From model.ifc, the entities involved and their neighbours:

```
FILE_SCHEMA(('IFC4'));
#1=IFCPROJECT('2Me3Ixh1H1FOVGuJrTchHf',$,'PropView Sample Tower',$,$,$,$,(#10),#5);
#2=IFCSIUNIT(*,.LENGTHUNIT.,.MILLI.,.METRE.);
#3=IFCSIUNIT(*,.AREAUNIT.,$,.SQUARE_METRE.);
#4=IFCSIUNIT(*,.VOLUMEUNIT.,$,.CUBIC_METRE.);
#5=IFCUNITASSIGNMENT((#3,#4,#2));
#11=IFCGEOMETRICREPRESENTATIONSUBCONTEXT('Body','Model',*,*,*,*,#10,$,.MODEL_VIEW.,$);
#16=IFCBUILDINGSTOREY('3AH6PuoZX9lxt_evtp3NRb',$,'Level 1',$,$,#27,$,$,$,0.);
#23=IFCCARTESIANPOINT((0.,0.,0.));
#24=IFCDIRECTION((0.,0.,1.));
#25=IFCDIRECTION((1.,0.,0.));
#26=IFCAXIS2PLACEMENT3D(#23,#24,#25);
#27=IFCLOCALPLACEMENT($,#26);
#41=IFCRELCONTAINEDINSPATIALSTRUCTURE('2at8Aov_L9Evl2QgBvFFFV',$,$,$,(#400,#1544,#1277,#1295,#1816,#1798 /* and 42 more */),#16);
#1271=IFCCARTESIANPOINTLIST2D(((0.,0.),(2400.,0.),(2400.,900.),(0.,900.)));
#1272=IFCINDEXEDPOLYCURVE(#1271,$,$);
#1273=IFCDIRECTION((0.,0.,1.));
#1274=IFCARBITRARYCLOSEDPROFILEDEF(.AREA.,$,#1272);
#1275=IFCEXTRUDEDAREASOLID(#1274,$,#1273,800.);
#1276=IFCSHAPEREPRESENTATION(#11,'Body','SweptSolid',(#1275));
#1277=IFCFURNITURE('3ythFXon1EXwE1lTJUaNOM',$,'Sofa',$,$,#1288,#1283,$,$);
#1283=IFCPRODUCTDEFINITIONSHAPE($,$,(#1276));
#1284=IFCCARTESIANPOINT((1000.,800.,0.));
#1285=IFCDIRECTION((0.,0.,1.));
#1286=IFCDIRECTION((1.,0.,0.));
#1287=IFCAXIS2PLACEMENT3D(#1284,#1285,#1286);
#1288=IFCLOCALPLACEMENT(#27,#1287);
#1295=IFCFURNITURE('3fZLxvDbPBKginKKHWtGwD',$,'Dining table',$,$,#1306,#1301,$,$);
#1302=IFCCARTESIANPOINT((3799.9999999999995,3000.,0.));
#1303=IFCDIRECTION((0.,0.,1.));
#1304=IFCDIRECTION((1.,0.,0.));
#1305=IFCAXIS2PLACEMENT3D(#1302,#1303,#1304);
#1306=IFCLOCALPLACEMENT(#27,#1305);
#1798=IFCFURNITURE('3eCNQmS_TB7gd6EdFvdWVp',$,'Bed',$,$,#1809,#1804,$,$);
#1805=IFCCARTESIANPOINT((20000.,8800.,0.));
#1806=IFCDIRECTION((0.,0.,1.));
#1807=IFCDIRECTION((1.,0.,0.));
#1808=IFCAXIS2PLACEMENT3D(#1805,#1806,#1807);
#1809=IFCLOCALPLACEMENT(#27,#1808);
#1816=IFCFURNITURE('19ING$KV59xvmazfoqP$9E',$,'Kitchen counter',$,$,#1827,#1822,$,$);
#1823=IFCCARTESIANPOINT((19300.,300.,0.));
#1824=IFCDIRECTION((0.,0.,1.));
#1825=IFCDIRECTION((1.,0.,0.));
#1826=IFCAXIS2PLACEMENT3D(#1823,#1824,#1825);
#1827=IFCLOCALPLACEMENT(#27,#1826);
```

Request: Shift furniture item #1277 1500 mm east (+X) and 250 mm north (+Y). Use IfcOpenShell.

```python
import ifcopenshell
import ifcopenshell.api.geometry
import ifcopenshell.util.placement

model = ifcopenshell.open("model.ifc")

item = model.by_guid("3ythFXon1EXwE1lTJUaNOM")
matrix = ifcopenshell.util.placement.get_local_placement(item.ObjectPlacement)
matrix[0, 3] += 1500.0
matrix[1, 3] += 250.0
ifcopenshell.api.geometry.edit_object_placement(model, product=item, matrix=matrix, is_si=False)

print(ifcopenshell.util.placement.get_local_placement(item.ObjectPlacement).round(3) + 0.0)

model.write("model_edited.ifc")
```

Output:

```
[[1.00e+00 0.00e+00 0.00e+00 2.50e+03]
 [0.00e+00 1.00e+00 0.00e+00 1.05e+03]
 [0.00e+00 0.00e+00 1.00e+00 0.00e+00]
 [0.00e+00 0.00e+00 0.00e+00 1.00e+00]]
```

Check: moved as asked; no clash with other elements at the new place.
